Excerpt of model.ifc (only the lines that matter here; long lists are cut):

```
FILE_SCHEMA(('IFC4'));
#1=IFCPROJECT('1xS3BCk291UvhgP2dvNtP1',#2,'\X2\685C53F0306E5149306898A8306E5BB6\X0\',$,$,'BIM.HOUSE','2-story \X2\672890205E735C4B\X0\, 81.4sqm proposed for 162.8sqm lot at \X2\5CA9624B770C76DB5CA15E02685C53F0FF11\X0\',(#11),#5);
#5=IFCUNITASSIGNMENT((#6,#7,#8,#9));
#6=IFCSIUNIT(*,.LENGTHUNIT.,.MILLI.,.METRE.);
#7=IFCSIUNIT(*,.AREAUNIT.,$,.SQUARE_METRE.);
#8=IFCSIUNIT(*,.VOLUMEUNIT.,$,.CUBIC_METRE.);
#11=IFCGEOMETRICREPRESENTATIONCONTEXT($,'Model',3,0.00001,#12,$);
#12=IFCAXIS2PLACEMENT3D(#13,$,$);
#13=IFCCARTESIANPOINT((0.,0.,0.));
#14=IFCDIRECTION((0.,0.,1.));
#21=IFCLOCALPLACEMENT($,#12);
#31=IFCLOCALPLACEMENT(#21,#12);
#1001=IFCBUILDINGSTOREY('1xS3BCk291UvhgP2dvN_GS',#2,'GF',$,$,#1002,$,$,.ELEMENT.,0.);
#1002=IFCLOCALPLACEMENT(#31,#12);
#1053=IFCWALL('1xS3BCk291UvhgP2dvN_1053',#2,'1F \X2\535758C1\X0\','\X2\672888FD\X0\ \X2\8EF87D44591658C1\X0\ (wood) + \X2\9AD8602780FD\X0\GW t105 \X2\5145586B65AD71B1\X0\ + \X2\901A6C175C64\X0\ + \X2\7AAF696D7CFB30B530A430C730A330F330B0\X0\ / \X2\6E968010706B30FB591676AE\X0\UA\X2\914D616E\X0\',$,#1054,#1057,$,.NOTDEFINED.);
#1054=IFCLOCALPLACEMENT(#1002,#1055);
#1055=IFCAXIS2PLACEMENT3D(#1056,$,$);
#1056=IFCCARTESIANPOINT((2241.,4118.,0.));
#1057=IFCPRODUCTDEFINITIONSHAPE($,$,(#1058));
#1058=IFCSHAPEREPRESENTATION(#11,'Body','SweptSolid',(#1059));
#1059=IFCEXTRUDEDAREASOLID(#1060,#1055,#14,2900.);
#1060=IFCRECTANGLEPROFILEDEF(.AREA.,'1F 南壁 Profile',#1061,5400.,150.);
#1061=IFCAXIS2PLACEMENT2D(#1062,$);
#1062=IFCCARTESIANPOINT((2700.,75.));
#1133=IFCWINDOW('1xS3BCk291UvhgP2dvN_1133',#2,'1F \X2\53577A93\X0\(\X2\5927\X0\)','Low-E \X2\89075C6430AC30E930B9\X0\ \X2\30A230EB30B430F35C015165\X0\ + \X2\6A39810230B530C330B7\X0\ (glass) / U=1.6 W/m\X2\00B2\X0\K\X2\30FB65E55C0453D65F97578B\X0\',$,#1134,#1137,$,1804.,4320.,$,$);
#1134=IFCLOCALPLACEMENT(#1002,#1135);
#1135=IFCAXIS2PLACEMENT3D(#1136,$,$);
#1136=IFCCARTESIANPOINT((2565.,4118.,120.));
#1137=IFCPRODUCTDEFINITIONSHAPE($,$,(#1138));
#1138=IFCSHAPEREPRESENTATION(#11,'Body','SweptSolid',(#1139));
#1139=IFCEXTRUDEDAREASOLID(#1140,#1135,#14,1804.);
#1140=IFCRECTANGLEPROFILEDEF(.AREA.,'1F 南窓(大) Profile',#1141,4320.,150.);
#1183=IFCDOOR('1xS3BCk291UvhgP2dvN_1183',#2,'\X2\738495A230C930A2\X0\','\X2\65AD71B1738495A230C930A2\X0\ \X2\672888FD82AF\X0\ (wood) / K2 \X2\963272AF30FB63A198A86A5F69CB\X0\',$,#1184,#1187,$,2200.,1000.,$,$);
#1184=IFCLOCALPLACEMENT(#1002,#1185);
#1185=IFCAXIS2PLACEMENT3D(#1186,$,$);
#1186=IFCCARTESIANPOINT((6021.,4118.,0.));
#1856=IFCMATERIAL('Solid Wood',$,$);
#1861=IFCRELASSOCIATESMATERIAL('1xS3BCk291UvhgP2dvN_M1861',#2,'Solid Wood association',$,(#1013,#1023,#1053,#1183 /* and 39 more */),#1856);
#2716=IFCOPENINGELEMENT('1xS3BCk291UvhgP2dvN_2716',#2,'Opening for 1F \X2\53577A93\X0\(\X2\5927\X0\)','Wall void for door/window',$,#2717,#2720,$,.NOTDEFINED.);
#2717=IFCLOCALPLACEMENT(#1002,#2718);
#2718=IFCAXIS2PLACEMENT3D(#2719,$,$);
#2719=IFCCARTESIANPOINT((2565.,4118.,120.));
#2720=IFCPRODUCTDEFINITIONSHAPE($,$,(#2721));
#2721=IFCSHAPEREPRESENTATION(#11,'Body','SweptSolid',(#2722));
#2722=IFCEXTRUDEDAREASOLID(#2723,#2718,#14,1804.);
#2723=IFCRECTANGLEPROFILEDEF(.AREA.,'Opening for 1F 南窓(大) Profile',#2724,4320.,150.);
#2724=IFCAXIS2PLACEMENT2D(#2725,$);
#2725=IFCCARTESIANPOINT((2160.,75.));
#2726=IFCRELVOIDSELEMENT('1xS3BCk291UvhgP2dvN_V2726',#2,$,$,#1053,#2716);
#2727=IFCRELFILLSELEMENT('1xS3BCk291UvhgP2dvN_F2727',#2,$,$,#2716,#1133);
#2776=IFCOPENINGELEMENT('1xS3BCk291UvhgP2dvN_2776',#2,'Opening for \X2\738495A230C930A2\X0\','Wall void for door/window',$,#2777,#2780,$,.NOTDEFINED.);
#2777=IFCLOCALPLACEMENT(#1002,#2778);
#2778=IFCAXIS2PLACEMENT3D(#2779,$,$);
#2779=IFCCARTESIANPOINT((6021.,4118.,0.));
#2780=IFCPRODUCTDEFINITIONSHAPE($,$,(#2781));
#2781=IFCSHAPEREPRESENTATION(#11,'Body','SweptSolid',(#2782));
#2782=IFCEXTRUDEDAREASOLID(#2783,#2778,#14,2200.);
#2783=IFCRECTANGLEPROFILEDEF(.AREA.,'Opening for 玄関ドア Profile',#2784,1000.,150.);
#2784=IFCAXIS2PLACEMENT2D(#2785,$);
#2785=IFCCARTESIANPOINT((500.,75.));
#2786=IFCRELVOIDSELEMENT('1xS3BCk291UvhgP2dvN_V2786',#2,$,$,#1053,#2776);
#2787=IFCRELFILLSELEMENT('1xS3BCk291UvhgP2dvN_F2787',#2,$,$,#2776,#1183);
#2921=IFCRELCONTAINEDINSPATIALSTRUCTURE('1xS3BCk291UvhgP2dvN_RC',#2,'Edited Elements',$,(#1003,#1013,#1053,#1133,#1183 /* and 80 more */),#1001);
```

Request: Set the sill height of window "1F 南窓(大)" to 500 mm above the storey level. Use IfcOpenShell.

```python
import numpy as np
import ifcopenshell
import ifcopenshell.api.geometry
import ifcopenshell.geom
import ifcopenshell.util.element
import ifcopenshell.util.placement
import ifcopenshell.util.shape
import ifcopenshell.util.unit

model = ifcopenshell.open("model.ifc")
unit_scale = ifcopenshell.util.unit.calculate_unit_scale(model)

window = model.by_guid("1xS3BCk291UvhgP2dvN_1133")
opening = window.FillsVoids[0].RelatingOpeningElement
storey = ifcopenshell.util.element.get_container(window, ifc_class="IfcBuildingStorey")
level = ifcopenshell.util.placement.get_local_placement(storey.ObjectPlacement)[2, 3]

# The opening's origin need not be at the sill, so measure its lowest point.
shape = ifcopenshell.geom.create_shape(ifcopenshell.geom.settings(), opening)
bottom = ifcopenshell.util.shape.get_shape_bottom_elevation(shape, shape.geometry) / unit_scale
dz = level + 0.5 / unit_scale - bottom

shift = np.array([0.0, 0.0, dz])
# The window is not placed relative to its opening, so move both.
for product in (opening, window):
    matrix = ifcopenshell.util.placement.get_local_placement(product.ObjectPlacement)
    matrix[:3, 3] += shift
    ifcopenshell.api.geometry.edit_object_placement(model, product=product, matrix=matrix, is_si=False)

print(f"moved by {dz * unit_scale:+.3f} m")

model.write("model-out.ifc")
```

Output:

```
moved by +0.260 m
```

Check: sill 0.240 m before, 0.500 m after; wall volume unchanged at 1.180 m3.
